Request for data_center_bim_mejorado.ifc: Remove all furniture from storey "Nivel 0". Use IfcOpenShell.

First a look at what the model holds.

```python
import ifcopenshell
import ifcopenshell.util.element

model = ifcopenshell.open("data_center_bim_mejorado.ifc")
print(model.schema)
storey = next(s for s in model.by_type("IfcBuildingStorey") if s.Name == "Nivel 0")
furniture = [e for e in ifcopenshell.util.element.get_decomposition(storey) if e.is_a("IfcFurnishingElement")]
seen = {}
for e in furniture:
    element_type = ifcopenshell.util.element.get_type(e)
    name = element_type.Name if element_type not in (None, e) else None
    seen[name] = seen.get(name, 0) + 1
for name, count in sorted(seen.items(), key=str):
    print(count, "x", name)
```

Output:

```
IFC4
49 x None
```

```python
import ifcopenshell
import ifcopenshell.api.root
import ifcopenshell.util.element

model = ifcopenshell.open("data_center_bim_mejorado.ifc")

storey = next(s for s in model.by_type("IfcBuildingStorey") if s.Name == "Nivel 0")
furniture = [e for e in ifcopenshell.util.element.get_decomposition(storey) if e.is_a("IfcFurnishingElement")]

for e in furniture:
    ifcopenshell.api.root.remove_product(model, product=e)
print(len(furniture), "removed")

model.write("data_center_bim_mejorado_updated.ifc")
```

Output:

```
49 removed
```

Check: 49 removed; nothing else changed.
